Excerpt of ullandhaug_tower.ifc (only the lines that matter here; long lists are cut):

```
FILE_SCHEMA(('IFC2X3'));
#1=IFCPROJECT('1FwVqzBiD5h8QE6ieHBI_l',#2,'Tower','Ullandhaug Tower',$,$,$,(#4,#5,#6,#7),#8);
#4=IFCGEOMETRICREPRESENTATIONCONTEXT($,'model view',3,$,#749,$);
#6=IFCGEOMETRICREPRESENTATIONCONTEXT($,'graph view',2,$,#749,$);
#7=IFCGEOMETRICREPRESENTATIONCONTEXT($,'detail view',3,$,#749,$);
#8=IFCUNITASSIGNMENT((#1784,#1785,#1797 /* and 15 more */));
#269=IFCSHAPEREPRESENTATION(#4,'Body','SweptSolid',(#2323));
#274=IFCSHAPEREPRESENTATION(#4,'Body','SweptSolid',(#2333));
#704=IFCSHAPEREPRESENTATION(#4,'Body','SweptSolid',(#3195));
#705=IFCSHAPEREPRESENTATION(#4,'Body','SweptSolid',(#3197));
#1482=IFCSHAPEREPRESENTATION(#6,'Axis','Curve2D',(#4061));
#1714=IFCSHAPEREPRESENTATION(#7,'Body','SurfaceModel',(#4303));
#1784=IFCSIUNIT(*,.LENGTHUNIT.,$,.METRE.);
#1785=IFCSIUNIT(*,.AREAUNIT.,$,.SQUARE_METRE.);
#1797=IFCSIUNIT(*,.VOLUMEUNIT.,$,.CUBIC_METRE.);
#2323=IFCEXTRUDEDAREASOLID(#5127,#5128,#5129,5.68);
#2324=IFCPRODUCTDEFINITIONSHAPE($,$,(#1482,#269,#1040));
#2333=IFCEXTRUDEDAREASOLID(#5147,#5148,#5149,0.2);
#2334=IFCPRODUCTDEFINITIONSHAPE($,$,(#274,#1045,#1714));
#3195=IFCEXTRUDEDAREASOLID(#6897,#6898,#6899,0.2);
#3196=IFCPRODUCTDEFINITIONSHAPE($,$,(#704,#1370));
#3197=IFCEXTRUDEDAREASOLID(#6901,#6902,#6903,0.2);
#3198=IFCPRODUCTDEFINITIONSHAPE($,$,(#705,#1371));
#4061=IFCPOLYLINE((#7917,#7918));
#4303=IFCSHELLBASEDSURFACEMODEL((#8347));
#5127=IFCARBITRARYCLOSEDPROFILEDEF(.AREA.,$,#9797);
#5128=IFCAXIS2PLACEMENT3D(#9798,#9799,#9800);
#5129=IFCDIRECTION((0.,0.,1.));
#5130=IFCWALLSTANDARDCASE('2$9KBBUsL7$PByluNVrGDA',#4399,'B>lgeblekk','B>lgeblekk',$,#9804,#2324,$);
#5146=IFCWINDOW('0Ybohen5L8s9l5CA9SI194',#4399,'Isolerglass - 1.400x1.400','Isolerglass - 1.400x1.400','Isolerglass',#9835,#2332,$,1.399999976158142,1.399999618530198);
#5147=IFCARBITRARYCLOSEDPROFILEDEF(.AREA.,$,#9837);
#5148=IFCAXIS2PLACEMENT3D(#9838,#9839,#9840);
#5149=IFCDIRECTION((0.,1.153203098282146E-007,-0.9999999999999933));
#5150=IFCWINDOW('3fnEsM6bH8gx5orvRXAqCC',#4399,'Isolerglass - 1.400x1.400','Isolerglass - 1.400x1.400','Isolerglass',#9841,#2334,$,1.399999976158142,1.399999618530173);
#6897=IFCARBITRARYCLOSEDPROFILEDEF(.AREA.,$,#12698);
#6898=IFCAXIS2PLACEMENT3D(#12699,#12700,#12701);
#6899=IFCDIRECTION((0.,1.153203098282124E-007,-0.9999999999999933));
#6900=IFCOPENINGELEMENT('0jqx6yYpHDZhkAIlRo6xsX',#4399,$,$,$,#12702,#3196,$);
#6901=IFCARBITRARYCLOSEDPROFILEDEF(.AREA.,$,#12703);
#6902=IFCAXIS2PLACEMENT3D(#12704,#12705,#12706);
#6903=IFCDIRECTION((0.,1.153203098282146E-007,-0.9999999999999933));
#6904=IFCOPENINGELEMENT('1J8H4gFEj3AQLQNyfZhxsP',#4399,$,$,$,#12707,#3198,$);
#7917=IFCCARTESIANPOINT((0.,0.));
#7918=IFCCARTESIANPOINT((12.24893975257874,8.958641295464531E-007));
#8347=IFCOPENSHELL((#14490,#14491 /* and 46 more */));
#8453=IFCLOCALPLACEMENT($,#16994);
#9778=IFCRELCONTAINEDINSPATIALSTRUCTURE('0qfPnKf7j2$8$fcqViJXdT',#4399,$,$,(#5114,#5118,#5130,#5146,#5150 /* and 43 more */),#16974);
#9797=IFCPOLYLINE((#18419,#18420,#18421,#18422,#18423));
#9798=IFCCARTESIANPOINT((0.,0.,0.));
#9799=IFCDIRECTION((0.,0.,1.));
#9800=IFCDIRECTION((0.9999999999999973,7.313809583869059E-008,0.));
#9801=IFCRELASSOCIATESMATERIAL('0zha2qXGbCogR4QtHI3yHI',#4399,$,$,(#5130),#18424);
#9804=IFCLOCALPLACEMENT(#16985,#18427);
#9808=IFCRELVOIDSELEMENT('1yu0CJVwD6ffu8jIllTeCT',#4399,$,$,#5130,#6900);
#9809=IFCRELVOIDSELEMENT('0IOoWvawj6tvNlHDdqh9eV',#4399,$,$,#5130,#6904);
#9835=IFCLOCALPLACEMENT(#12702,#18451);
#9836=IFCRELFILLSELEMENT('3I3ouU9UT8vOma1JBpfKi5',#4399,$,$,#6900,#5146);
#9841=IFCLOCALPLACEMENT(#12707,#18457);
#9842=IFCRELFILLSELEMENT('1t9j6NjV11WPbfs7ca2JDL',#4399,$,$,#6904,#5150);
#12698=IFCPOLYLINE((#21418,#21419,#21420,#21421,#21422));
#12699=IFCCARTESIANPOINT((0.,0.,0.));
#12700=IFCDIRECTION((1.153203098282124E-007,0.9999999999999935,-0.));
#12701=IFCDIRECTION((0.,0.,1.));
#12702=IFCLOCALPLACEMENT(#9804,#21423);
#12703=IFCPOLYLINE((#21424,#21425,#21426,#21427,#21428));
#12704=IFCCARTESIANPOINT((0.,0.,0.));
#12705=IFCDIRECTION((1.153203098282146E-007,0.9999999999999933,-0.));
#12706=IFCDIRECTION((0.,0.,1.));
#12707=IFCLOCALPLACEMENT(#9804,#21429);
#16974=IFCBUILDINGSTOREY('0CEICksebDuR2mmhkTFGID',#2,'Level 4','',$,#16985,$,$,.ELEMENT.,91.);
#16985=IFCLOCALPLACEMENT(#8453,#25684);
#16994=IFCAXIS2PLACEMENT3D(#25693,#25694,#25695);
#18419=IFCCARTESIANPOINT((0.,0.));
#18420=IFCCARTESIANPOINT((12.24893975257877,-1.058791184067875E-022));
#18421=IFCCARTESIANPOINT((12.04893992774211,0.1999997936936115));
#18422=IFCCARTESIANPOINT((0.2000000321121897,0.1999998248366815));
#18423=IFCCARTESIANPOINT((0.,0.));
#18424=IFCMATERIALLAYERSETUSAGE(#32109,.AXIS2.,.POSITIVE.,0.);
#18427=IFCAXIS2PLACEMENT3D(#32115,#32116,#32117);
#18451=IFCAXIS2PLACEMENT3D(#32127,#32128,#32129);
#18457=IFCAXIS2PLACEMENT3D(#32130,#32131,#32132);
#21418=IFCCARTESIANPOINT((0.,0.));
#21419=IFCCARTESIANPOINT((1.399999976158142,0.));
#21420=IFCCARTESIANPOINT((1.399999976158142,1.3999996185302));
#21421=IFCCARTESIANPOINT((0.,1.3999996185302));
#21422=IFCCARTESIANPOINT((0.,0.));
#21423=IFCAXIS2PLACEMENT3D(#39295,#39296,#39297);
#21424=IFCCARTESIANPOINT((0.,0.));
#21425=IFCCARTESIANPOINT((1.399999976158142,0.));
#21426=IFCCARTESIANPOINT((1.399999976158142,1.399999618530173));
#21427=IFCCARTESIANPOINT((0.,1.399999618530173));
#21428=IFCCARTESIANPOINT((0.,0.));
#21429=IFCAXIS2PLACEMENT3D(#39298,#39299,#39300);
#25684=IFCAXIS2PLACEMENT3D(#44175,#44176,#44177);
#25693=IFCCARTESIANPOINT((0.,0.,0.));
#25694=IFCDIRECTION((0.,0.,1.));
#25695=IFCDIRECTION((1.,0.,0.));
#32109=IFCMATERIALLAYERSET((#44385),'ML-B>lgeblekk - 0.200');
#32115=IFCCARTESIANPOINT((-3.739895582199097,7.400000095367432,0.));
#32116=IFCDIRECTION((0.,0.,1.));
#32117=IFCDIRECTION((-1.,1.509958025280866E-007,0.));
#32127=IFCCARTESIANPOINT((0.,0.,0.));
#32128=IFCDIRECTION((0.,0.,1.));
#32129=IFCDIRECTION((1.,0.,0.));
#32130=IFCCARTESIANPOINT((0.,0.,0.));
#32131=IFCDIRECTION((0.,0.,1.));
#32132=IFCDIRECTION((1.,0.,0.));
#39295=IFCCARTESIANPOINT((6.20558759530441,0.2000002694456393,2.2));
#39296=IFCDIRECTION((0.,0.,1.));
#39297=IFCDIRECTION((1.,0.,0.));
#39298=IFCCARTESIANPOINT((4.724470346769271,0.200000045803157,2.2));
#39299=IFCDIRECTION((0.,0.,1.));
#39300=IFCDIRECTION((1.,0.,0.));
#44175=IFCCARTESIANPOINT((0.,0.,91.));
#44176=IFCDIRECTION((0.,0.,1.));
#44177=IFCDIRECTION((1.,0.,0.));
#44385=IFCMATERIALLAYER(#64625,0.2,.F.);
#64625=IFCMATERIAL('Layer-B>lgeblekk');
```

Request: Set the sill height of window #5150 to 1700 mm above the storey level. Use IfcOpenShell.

```python
import numpy as np
import ifcopenshell
import ifcopenshell.api.geometry
import ifcopenshell.geom
import ifcopenshell.util.element
import ifcopenshell.util.placement
import ifcopenshell.util.shape
import ifcopenshell.util.unit

model = ifcopenshell.open("ullandhaug_tower.ifc")
unit_scale = ifcopenshell.util.unit.calculate_unit_scale(model)

window = model.by_guid("3fnEsM6bH8gx5orvRXAqCC")
opening = window.FillsVoids[0].RelatingOpeningElement
storey = ifcopenshell.util.element.get_container(window, ifc_class="IfcBuildingStorey")
level = ifcopenshell.util.placement.get_local_placement(storey.ObjectPlacement)[2, 3]

# The opening's origin need not be at the sill, so measure its lowest point.
shape = ifcopenshell.geom.create_shape(ifcopenshell.geom.settings(), opening)
bottom = ifcopenshell.util.shape.get_shape_bottom_elevation(shape, shape.geometry) / unit_scale
dz = level + 1.7 - bottom

shift = np.array([0.0, 0.0, dz])
# The window is placed relative to its opening, so it follows when the opening moves.
matrix = ifcopenshell.util.placement.get_local_placement(opening.ObjectPlacement)
matrix[:3, 3] += shift
ifcopenshell.api.geometry.edit_object_placement(
    model, product=opening, matrix=matrix, is_si=False, should_transform_children=True
)

print(f"moved by {dz * unit_scale:+.3f} m")

model.write("ullandhaug_tower_updated.ifc")
```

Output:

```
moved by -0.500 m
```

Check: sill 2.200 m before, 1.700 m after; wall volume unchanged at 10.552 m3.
